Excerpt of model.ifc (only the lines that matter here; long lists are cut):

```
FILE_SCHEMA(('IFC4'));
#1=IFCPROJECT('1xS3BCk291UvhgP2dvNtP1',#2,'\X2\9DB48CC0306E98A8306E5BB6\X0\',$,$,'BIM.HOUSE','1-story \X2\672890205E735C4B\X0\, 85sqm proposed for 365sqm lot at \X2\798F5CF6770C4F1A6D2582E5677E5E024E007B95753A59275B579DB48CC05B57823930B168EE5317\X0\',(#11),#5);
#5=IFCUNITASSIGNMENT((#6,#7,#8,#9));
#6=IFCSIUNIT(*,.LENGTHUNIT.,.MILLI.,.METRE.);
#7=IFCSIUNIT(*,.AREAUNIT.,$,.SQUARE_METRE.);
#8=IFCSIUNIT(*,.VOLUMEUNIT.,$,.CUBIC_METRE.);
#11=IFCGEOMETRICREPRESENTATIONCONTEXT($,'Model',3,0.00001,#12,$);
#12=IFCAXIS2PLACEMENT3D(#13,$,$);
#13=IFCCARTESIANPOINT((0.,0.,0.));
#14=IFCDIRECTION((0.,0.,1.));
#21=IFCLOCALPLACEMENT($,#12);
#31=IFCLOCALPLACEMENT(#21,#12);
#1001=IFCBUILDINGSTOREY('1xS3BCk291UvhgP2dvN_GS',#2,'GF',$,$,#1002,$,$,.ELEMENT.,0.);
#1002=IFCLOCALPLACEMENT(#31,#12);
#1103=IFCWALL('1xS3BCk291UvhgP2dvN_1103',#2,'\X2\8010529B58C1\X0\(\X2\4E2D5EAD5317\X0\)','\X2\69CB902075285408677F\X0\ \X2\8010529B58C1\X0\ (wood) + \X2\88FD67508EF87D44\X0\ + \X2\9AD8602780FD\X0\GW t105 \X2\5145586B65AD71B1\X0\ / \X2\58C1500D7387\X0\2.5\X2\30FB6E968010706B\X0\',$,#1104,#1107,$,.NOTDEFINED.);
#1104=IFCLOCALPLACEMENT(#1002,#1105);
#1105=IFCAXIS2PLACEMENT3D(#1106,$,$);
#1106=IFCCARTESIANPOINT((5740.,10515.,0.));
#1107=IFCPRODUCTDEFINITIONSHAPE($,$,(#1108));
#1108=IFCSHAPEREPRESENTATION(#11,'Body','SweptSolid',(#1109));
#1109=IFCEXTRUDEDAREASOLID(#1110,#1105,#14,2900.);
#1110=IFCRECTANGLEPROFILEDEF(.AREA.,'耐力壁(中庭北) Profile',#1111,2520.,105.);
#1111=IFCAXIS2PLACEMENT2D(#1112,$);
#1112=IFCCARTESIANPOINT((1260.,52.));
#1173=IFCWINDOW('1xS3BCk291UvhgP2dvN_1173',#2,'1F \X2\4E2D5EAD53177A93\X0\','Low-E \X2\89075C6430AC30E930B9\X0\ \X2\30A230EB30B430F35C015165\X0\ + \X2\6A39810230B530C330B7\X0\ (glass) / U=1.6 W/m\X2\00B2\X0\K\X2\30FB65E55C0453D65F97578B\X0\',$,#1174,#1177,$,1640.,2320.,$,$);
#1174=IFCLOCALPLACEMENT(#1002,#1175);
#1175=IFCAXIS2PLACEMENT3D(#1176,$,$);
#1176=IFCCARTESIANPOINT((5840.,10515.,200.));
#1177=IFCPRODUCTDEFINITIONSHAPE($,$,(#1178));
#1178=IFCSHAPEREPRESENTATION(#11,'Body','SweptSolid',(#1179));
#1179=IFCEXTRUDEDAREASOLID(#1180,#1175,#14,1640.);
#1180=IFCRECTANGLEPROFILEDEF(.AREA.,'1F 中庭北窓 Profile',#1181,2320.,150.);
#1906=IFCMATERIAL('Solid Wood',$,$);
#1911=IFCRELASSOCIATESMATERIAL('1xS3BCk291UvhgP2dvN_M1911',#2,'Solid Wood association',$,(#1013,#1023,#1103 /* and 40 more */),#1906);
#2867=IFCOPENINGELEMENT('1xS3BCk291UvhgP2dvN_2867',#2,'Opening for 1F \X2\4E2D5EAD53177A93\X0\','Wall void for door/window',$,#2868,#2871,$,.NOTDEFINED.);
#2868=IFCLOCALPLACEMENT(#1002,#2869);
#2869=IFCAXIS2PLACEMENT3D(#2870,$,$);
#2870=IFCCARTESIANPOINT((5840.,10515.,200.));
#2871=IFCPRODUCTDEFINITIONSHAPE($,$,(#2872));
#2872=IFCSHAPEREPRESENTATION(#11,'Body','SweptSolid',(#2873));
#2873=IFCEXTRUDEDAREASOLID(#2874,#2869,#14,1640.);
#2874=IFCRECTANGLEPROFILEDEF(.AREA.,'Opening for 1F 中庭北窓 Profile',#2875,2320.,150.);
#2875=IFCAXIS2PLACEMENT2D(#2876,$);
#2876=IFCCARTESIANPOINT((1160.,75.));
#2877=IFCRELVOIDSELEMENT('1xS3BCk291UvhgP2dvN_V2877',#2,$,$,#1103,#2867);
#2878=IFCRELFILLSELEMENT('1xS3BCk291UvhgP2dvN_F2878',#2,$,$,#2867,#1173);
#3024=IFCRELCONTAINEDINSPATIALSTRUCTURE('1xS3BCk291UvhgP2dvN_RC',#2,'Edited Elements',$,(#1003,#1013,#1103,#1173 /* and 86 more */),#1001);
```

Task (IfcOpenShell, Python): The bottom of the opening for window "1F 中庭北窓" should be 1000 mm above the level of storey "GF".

```python
import numpy as np
import ifcopenshell
import ifcopenshell.api.geometry
import ifcopenshell.geom
import ifcopenshell.util.element
import ifcopenshell.util.placement
import ifcopenshell.util.shape
import ifcopenshell.util.unit

model = ifcopenshell.open("model.ifc")
unit_scale = ifcopenshell.util.unit.calculate_unit_scale(model)

window = model.by_guid("1xS3BCk291UvhgP2dvN_1173")
opening = window.FillsVoids[0].RelatingOpeningElement
storey = ifcopenshell.util.element.get_container(window, ifc_class="IfcBuildingStorey")
level = ifcopenshell.util.placement.get_local_placement(storey.ObjectPlacement)[2, 3]

# The opening's origin need not be at the sill, so measure its lowest point.
shape = ifcopenshell.geom.create_shape(ifcopenshell.geom.settings(), opening)
bottom = ifcopenshell.util.shape.get_shape_bottom_elevation(shape, shape.geometry) / unit_scale
dz = level + 1 / unit_scale - bottom

shift = np.array([0.0, 0.0, dz])
# The window is not placed relative to its opening, so move both.
for product in (opening, window):
    matrix = ifcopenshell.util.placement.get_local_placement(product.ObjectPlacement)
    matrix[:3, 3] += shift
    ifcopenshell.api.geometry.edit_object_placement(model, product=product, matrix=matrix, is_si=False)

print(f"moved by {dz * unit_scale:+.3f} m")

model.write("model-out.ifc")
```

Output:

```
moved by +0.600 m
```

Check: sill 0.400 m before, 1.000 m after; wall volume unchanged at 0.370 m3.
